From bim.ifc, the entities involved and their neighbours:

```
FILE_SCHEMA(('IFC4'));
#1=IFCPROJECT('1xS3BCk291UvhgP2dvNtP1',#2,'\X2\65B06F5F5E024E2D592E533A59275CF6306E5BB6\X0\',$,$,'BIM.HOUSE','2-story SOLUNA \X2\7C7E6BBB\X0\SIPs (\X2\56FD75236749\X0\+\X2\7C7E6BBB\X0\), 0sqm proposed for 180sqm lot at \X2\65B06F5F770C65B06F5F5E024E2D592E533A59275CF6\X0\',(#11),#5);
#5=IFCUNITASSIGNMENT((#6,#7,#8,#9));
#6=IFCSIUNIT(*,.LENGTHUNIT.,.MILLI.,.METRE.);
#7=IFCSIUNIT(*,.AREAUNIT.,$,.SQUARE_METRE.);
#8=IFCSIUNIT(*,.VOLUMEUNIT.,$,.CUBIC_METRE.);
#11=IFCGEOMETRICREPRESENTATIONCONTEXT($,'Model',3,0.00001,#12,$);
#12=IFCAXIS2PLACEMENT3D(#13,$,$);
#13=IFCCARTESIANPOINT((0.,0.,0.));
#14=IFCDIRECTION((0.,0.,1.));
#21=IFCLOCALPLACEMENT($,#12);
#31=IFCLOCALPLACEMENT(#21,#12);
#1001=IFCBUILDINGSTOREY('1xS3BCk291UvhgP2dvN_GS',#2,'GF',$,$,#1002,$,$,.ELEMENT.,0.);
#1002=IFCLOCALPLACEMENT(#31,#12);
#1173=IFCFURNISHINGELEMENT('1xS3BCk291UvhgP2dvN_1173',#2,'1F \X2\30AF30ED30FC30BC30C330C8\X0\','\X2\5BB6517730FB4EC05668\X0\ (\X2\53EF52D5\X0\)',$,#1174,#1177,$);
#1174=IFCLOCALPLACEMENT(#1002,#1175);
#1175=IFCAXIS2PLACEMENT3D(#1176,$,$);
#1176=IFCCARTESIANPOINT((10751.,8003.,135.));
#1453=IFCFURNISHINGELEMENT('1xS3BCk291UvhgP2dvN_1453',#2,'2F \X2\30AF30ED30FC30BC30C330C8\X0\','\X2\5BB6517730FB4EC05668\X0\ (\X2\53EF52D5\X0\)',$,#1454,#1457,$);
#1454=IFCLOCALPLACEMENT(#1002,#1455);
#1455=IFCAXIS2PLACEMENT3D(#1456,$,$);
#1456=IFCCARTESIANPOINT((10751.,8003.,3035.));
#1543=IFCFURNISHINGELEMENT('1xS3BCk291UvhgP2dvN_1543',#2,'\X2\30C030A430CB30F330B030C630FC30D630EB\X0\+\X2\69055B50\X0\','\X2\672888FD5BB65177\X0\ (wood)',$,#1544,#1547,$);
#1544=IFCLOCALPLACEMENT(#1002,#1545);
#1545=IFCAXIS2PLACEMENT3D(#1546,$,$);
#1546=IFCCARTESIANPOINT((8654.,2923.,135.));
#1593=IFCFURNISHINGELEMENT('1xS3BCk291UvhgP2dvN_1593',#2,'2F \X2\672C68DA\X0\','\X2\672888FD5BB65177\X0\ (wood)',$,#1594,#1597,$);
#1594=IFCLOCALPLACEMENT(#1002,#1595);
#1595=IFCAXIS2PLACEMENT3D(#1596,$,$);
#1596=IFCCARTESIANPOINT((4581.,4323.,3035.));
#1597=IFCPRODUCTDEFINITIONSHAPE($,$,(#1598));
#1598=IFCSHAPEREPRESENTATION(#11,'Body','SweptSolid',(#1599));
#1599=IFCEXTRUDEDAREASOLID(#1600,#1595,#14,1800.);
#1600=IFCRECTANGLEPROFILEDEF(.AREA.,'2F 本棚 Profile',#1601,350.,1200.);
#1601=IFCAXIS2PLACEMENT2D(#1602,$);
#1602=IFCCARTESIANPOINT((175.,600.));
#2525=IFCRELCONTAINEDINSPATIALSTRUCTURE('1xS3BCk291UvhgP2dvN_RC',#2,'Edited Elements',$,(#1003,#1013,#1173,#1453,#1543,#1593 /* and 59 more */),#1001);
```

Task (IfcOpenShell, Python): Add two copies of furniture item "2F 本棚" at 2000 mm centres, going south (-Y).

```python
import numpy as np
import ifcopenshell
import ifcopenshell.api.geometry
import ifcopenshell.api.root
import ifcopenshell.util.element
import ifcopenshell.util.placement
import ifcopenshell.util.unit

model = ifcopenshell.open("bim.ifc")
unit_scale = ifcopenshell.util.unit.calculate_unit_scale(model)


def reuse_history(source, copy):
    """copy_class also copies each property set's owner history, people and application; keep the originals."""
    for rel in copy.IsDefinedBy:
        if rel.is_a("IfcRelDefinesByProperties") and (history := rel.RelatingPropertyDefinition.OwnerHistory):
            rel.RelatingPropertyDefinition.OwnerHistory = source.OwnerHistory
            ifcopenshell.util.element.remove_deep2(model, history)


source = model.by_guid("1xS3BCk291UvhgP2dvN_1593")
base = ifcopenshell.util.placement.get_local_placement(source.ObjectPlacement)
step = np.array([0.0, -1.0, 0.0]) * 2 / unit_scale

for i in range(1, 3):
    copy = ifcopenshell.api.root.copy_class(model, product=source)
    copy.Representation = ifcopenshell.util.element.copy_deep(
        model, source.Representation, exclude=["IfcGeometricRepresentationContext", "IfcRepresentationMap"]
    )
    reuse_history(source, copy)
    matrix = base.copy()
    matrix[:3, 3] += i * step
    print("added at", matrix[:3, 3].round(3) + 0.0)
    ifcopenshell.api.geometry.edit_object_placement(model, product=copy, matrix=matrix, is_si=False)

model.write("bim_v2.ifc")
```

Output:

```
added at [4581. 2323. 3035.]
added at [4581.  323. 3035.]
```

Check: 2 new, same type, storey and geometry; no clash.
